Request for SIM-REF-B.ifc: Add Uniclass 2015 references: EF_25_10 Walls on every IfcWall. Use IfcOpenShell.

First a look at what the model holds.

```python
import ifcopenshell

model = ifcopenshell.open("SIM-REF-B.ifc")
print(model.schema)
print("classifications:", [c.Name for c in model.by_type("IfcClassification")])
for ifc_class in ("IfcDoor", "IfcRoof", "IfcStair", "IfcWall", "IfcWindow"):
    print(ifc_class, len(model.by_type(ifc_class)))
```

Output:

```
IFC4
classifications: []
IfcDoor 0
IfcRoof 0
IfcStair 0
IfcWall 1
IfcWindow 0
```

```python
import ifcopenshell
import ifcopenshell.api.classification

model = ifcopenshell.open("SIM-REF-B.ifc")

system = ifcopenshell.api.classification.add_classification(model, classification="Uniclass 2015")

codes = {
    "IfcWall": ("EF_25_10", "Walls"),
}
for ifc_class, (code, name) in codes.items():
    products = model.by_type(ifc_class)
    ifcopenshell.api.classification.add_reference(
        model, products=products, classification=system, identification=code, name=name
    )
    print(code, len(products))

model.write("SIM-REF-B_edited.ifc")
```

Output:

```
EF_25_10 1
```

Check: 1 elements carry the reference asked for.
